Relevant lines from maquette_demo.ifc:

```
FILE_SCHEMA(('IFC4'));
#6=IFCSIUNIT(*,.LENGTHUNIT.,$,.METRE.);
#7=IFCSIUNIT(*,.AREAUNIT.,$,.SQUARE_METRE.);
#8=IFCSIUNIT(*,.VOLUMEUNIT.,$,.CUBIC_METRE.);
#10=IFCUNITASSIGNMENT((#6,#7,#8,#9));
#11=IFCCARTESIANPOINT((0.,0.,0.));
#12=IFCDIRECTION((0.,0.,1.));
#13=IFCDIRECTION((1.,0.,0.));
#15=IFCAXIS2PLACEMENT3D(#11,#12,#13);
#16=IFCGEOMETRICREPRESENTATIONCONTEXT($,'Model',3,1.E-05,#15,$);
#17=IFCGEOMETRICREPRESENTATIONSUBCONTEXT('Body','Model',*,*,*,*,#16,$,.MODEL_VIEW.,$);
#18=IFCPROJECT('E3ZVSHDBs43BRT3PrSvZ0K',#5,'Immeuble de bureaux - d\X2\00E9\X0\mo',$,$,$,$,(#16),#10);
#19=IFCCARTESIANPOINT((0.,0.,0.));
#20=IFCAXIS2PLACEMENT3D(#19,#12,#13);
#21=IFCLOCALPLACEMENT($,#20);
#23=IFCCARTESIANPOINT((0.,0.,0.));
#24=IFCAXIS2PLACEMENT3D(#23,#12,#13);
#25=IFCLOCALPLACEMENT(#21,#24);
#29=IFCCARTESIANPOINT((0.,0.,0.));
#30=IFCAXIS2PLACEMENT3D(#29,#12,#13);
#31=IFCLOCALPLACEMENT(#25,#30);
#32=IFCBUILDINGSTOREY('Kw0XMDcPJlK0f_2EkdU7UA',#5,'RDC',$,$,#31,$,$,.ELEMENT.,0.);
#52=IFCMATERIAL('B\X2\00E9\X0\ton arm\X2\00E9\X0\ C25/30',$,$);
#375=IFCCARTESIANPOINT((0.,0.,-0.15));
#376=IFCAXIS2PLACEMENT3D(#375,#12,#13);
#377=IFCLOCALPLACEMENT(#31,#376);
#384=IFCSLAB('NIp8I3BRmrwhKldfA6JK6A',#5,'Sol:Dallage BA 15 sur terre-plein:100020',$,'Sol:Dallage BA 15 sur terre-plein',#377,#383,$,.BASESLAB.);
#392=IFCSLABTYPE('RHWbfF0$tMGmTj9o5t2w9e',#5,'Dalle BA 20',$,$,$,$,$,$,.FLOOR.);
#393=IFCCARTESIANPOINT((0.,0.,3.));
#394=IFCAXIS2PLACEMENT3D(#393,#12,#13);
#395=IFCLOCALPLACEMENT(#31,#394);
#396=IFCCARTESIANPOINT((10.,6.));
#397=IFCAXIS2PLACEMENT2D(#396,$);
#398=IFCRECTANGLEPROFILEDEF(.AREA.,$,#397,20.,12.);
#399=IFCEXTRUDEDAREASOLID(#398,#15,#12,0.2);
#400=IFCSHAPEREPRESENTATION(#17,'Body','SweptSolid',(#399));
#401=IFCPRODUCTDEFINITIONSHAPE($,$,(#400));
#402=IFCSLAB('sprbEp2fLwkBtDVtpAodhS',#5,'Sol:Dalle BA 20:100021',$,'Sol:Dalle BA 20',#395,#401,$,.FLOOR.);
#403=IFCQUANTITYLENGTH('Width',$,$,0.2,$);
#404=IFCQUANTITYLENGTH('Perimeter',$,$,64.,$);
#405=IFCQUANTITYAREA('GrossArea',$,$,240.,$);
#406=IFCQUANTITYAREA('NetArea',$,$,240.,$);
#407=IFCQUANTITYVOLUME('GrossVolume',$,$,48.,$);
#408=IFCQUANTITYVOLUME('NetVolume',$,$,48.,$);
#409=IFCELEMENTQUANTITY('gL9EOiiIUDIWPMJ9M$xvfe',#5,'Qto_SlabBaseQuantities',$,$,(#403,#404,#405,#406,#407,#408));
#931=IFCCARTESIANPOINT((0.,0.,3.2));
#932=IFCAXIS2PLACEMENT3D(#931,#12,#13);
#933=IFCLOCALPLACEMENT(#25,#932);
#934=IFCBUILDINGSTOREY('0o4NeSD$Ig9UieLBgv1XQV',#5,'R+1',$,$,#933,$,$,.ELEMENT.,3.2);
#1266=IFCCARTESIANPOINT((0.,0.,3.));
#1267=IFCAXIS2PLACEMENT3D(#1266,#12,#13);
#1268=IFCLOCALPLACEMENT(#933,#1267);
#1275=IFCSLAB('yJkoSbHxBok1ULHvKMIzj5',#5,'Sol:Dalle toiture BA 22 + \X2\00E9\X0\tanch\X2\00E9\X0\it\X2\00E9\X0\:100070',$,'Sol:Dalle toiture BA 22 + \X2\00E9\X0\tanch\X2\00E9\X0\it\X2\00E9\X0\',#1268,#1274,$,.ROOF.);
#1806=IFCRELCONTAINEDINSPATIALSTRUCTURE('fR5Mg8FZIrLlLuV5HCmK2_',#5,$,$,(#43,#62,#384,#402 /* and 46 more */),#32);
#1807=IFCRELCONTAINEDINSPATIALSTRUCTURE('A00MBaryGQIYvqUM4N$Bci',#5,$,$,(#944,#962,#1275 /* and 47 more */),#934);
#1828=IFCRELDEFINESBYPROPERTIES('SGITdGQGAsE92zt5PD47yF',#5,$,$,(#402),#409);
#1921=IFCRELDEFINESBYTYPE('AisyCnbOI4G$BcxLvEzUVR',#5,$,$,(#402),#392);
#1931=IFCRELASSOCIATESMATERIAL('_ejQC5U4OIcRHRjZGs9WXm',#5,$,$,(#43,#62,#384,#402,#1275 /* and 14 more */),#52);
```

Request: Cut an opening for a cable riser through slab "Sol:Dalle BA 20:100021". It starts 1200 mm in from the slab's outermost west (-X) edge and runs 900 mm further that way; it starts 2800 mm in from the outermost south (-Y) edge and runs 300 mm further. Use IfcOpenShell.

```python
import numpy as np
import ifcopenshell
import ifcopenshell.api.feature
import ifcopenshell.api.geometry
import ifcopenshell.api.pset
import ifcopenshell.api.root
import ifcopenshell.geom
import ifcopenshell.util.element
import ifcopenshell.util.placement
import ifcopenshell.util.representation
import ifcopenshell.util.shape
import ifcopenshell.util.unit

model = ifcopenshell.open("maquette_demo.ifc")
unit_scale = ifcopenshell.util.unit.calculate_unit_scale(model)
area_scale = ifcopenshell.util.unit.calculate_unit_scale(model, "AREAUNIT")
volume_scale = ifcopenshell.util.unit.calculate_unit_scale(model, "VOLUMEUNIT")
settings = ifcopenshell.geom.settings()


def volume(element):
    """Net volume in cubic metres, openings subtracted."""
    shape = ifcopenshell.geom.create_shape(settings, element)
    return ifcopenshell.util.shape.get_volume(shape.geometry)


slab = model.by_id(402)
before = volume(slab)

# Extent in the slab's own axes, in metres. The edges named are its -X and -Y sides.
slab_shape = ifcopenshell.geom.create_shape(settings, slab)
vertices = ifcopenshell.util.shape.get_vertices(slab_shape.geometry)
x_min, y_min, bottom = vertices.min(axis=0)
top = vertices[:, 2].max()

opening = ifcopenshell.api.root.create_entity(model, ifc_class="IfcOpeningElement", name="Cable riser opening", predefined_type="OPENING")
context = ifcopenshell.util.representation.get_context(model, "Model", "Body", "MODEL_VIEW")
width, depth = 0.9, 0.3
outline = [(0.0, 0.0), (width, 0.0), (width, depth), (0.0, depth), (0.0, 0.0)]
# Overshoot both faces by 50 mm so the cut is clean.
shape = ifcopenshell.api.geometry.add_slab_representation(
    model, context=context, depth=top - bottom + 0.1, polyline=outline
)
ifcopenshell.api.geometry.assign_representation(model, product=opening, representation=shape)

matrix = ifcopenshell.util.placement.get_local_placement(slab.ObjectPlacement)
matrix[:, 3] = matrix @ np.append(np.array([x_min + 1.2, y_min + 2.8, bottom - 0.05]) / unit_scale, 1.0)
ifcopenshell.api.geometry.edit_object_placement(model, product=opening, matrix=matrix, is_si=False)
ifcopenshell.api.feature.add_feature(model, feature=opening, element=slab)

after = volume(slab)

# Update the slab's stored quantities.
qto = model.by_id(ifcopenshell.util.element.get_pset(slab, "Qto_SlabBaseQuantities", should_inherit=False)["id"])
ifcopenshell.api.pset.edit_qto(model, qto=qto, properties={
    "NetArea": after / (top - bottom) / area_scale,
    "NetVolume": after / volume_scale,
})

print(f"slab volume {before:.3f} -> {after:.3f} m3")

model.write("maquette_demo_updated.ifc")
```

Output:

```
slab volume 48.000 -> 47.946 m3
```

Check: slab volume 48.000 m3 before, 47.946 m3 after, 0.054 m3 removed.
